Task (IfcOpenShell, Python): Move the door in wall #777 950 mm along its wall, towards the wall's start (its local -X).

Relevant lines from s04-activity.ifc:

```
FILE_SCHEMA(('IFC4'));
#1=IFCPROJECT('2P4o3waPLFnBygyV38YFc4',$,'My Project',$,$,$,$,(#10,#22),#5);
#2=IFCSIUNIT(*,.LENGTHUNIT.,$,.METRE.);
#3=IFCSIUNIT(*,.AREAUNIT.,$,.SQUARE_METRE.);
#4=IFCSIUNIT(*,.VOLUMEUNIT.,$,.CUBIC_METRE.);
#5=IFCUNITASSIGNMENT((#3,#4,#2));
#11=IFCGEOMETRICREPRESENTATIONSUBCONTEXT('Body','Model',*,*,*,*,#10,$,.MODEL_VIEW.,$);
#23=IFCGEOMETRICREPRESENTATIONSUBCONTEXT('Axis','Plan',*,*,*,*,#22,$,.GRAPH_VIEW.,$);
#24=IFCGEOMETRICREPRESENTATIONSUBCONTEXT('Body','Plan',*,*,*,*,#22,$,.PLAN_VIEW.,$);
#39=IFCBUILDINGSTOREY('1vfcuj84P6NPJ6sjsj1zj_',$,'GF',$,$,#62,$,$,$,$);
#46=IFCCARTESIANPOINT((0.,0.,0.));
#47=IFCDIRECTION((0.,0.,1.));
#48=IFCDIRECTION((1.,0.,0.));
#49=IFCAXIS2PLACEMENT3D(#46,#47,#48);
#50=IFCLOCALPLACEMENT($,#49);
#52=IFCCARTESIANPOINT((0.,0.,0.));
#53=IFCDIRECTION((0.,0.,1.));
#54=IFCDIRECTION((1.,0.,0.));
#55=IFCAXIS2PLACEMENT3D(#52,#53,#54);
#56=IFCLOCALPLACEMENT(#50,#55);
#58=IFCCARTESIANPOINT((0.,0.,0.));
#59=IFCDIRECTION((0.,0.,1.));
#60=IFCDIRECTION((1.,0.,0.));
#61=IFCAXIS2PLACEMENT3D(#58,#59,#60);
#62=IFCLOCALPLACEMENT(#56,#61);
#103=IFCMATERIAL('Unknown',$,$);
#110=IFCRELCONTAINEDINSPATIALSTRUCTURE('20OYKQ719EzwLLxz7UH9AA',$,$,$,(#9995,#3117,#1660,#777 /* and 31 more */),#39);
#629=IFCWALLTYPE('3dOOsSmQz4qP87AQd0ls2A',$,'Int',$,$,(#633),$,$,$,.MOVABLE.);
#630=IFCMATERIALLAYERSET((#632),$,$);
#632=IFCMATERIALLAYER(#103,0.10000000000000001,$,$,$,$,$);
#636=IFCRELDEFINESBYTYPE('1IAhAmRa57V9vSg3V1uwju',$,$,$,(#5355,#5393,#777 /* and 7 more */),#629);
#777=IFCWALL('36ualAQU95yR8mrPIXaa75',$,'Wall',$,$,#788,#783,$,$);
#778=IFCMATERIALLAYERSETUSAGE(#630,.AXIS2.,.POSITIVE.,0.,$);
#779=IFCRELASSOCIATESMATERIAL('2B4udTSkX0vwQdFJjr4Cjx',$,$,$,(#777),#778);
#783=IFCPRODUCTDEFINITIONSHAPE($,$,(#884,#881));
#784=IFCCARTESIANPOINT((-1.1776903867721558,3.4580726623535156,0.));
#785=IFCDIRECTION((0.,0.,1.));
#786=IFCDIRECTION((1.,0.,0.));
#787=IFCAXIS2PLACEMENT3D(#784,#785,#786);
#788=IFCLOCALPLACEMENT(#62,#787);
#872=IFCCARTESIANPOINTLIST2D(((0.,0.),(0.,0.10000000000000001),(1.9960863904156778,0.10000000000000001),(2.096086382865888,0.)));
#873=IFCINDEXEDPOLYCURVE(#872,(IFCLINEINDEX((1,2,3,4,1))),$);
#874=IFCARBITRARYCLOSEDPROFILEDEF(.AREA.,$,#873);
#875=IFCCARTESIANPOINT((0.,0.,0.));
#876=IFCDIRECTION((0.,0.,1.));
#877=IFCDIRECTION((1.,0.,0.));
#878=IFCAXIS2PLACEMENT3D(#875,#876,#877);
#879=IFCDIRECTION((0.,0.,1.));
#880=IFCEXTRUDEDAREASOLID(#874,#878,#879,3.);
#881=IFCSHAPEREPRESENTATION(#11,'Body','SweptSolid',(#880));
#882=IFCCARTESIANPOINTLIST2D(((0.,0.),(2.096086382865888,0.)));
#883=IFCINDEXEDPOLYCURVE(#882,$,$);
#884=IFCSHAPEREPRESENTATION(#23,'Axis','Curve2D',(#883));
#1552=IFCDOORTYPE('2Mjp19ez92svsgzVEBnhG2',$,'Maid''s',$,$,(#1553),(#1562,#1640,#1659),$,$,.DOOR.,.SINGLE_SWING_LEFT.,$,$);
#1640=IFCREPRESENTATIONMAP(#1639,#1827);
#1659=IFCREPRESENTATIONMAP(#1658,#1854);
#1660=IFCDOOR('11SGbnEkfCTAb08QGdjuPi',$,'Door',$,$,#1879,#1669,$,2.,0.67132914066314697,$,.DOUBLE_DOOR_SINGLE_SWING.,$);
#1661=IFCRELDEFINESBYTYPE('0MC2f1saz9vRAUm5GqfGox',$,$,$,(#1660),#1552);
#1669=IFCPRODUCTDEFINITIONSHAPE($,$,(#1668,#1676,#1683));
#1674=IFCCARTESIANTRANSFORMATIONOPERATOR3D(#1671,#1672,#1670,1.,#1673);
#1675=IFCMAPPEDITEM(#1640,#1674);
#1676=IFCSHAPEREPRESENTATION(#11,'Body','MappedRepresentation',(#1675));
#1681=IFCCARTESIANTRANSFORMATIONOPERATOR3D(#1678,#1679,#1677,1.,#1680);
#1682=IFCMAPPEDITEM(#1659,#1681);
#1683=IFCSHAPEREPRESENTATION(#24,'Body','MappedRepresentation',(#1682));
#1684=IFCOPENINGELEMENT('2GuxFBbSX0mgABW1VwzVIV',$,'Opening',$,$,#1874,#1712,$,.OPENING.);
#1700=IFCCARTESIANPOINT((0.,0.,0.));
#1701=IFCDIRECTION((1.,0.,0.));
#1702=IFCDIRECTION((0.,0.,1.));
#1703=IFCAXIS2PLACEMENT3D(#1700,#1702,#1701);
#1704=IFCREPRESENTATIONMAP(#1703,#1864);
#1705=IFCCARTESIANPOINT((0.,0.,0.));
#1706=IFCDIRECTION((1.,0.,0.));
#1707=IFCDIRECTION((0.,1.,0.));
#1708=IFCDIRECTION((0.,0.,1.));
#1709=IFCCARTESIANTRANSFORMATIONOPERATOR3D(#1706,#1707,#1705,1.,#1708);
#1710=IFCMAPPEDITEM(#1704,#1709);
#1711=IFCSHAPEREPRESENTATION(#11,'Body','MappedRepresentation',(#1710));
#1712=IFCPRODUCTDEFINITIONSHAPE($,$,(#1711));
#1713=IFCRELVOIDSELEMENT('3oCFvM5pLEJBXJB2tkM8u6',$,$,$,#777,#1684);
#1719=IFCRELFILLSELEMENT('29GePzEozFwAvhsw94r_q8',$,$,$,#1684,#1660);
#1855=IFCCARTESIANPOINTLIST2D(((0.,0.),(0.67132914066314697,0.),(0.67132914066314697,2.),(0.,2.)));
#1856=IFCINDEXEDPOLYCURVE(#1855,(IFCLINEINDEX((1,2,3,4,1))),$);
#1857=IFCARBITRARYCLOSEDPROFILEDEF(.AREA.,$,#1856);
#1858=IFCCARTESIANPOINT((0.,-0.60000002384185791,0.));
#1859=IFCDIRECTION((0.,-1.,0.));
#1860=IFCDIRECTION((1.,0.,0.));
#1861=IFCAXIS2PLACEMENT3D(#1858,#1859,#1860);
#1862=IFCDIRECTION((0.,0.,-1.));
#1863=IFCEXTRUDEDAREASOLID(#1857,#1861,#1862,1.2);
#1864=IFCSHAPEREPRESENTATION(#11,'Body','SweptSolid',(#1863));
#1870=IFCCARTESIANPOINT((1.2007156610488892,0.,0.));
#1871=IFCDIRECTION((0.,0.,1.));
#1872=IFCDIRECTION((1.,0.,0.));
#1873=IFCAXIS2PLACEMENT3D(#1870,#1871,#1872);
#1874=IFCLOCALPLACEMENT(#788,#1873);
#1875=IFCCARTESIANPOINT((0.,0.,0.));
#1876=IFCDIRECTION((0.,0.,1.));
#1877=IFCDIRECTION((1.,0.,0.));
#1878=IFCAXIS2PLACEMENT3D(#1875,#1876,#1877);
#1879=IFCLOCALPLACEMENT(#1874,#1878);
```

```python
import ifcopenshell
import ifcopenshell.api.geometry
import ifcopenshell.util.placement
import ifcopenshell.util.unit

model = ifcopenshell.open("s04-activity.ifc")
unit_scale = ifcopenshell.util.unit.calculate_unit_scale(model)

door = model.by_id(1660)
opening = door.FillsVoids[0].RelatingOpeningElement
wall = opening.VoidsElements[0].RelatingBuildingElement

wall_matrix = ifcopenshell.util.placement.get_local_placement(wall.ObjectPlacement)
shift = wall_matrix[:3, 0] * -0.95 / unit_scale
before = ifcopenshell.util.placement.get_local_placement(door.ObjectPlacement)[:3, 3].copy()

# The door is placed relative to its opening, so it follows when the opening moves.
matrix = ifcopenshell.util.placement.get_local_placement(opening.ObjectPlacement)
matrix[:3, 3] += shift
ifcopenshell.api.geometry.edit_object_placement(
    model, product=opening, matrix=matrix, is_si=False, should_transform_children=True
)

after = ifcopenshell.util.placement.get_local_placement(door.ObjectPlacement)[:3, 3]
print("door moved by", (after - before).round(3) + 0.0)

model.write("s04-activity_rev.ifc")
```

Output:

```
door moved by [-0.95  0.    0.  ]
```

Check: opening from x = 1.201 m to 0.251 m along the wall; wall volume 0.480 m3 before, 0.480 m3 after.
